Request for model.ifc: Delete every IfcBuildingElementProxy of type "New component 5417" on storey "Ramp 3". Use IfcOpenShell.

First a look at what the model holds.

```python
import ifcopenshell
import ifcopenshell.util.element

model = ifcopenshell.open("model.ifc")
print(model.schema)
storey = next(s for s in model.by_type("IfcBuildingStorey") if s.Name == "Ramp 3")
proxies = [e for e in ifcopenshell.util.element.get_decomposition(storey) if e.is_a("IfcBuildingElementProxy")]
seen = {}
for e in proxies:
    element_type = ifcopenshell.util.element.get_type(e)
    name = element_type.Name if element_type not in (None, e) else None
    seen[name] = seen.get(name, 0) + 1
for name, count in sorted(seen.items(), key=str):
    print(count, "x", name)
```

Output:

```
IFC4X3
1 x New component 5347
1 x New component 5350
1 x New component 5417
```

```python
import ifcopenshell
import ifcopenshell.api.root
import ifcopenshell.util.element

model = ifcopenshell.open("model.ifc")

storey = next(s for s in model.by_type("IfcBuildingStorey") if s.Name == "Ramp 3")
proxies = [e for e in ifcopenshell.util.element.get_decomposition(storey) if e.is_a("IfcBuildingElementProxy")]
targets = [e for e in proxies if (t := ifcopenshell.util.element.get_type(e)) not in (None, e) and t.Name == "New component 5417"]

for e in targets:
    ifcopenshell.api.root.remove_product(model, product=e)
print(len(targets), "removed")

model.write("model_edited.ifc")
```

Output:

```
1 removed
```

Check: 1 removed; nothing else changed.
